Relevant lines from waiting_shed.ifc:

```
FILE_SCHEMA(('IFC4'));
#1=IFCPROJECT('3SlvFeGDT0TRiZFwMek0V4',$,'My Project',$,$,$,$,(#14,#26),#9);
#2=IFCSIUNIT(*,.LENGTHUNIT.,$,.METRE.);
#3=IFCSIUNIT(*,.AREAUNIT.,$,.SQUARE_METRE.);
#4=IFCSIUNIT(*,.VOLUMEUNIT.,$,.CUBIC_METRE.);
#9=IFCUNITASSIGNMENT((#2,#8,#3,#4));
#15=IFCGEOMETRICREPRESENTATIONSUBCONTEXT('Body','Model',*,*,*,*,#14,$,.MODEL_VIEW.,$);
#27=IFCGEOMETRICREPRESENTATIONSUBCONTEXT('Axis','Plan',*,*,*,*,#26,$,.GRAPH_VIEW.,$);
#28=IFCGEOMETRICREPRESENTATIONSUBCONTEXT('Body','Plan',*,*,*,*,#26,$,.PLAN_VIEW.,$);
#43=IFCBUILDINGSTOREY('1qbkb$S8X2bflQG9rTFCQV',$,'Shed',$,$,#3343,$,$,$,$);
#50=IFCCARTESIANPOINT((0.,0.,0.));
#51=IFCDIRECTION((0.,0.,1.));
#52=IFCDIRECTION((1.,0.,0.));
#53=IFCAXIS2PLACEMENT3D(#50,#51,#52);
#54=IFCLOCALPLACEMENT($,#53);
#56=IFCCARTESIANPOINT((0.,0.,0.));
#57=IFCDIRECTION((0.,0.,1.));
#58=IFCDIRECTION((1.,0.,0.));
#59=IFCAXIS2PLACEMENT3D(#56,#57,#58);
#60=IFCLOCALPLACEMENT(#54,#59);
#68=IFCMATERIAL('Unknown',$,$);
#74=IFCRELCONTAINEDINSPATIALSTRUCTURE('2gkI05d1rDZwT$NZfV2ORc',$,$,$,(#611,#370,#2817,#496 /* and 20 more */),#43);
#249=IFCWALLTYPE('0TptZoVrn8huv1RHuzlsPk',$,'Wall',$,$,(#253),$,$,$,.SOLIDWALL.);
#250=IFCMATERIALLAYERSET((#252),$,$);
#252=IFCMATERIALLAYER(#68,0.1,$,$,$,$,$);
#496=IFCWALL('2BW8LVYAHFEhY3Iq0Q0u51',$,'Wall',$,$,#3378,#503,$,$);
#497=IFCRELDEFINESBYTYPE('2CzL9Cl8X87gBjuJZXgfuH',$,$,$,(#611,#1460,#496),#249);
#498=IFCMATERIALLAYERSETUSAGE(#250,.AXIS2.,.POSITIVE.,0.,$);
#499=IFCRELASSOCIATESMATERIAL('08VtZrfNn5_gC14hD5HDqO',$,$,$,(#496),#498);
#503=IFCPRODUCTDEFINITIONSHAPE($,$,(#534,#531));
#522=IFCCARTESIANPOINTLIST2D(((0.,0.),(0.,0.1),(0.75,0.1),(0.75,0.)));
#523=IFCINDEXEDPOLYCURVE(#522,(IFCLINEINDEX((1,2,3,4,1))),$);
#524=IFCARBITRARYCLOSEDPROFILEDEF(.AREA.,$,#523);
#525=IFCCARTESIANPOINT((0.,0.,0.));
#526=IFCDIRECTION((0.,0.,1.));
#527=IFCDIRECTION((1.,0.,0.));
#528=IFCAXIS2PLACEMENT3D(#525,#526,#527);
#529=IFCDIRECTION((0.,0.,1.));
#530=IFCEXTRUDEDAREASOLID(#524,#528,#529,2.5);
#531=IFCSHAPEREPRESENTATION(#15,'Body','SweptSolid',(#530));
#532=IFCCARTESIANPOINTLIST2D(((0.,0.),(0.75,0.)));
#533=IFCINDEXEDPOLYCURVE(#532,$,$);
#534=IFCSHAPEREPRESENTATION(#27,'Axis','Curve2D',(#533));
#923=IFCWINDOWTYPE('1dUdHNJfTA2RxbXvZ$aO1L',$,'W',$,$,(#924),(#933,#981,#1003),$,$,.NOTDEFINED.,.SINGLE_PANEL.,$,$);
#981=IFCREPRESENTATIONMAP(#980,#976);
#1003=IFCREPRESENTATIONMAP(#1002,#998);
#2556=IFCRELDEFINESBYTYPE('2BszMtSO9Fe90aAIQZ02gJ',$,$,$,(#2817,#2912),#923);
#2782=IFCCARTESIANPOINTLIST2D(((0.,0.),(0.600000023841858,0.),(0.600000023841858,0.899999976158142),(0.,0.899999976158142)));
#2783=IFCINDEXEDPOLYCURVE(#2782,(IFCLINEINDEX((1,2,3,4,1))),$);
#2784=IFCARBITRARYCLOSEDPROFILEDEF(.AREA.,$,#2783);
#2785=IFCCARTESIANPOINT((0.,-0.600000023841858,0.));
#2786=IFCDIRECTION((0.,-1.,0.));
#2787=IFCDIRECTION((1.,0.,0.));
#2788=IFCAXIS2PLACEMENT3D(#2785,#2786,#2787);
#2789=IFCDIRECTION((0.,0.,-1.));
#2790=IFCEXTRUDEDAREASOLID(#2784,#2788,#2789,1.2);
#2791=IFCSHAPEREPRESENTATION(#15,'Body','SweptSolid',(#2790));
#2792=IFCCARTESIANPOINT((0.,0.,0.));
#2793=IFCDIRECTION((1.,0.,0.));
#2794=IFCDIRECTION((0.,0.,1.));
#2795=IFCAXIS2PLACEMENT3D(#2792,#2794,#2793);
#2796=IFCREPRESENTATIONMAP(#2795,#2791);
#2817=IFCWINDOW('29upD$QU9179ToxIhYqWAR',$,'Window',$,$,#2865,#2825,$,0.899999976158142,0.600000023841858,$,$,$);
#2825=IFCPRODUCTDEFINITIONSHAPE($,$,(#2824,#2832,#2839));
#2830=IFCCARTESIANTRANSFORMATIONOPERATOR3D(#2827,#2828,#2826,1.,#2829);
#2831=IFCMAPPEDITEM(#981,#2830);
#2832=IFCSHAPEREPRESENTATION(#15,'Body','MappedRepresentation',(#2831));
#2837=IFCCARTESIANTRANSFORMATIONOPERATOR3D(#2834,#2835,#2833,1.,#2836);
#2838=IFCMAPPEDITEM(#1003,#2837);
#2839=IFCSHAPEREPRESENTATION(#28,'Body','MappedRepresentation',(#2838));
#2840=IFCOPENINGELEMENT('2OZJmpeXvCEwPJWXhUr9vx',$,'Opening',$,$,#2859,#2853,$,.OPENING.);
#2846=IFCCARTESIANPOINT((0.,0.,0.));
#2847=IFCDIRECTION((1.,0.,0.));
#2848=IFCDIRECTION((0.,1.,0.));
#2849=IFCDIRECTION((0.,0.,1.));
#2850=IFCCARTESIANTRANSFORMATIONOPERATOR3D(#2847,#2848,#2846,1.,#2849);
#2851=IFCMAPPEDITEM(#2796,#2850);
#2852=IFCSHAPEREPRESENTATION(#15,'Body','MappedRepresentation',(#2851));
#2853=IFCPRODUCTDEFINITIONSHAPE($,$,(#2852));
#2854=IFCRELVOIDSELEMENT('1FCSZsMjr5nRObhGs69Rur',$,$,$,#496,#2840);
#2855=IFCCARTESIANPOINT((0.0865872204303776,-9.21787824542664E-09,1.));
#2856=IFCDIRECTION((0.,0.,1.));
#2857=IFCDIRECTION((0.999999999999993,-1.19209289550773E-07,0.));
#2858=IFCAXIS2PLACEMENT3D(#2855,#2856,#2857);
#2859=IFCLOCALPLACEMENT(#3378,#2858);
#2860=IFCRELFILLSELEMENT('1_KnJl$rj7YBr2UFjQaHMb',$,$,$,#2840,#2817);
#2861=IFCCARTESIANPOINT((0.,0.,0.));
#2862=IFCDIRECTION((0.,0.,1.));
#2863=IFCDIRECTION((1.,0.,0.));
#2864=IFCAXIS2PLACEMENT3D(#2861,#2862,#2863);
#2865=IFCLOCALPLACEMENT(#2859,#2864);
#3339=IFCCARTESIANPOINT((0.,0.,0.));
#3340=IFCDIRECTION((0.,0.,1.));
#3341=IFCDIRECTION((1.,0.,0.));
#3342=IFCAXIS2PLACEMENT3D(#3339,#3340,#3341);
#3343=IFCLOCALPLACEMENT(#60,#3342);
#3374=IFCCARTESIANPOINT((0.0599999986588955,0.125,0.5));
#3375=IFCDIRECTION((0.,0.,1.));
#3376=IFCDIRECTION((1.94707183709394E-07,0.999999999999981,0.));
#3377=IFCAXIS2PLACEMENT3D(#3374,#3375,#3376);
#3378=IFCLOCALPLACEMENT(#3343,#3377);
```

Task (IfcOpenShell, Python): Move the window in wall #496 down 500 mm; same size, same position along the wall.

```python
import numpy as np
import ifcopenshell
import ifcopenshell.api.geometry
import ifcopenshell.util.placement
import ifcopenshell.util.unit

model = ifcopenshell.open("waiting_shed.ifc")
unit_scale = ifcopenshell.util.unit.calculate_unit_scale(model)

window = model.by_id(2817)
opening = window.FillsVoids[0].RelatingOpeningElement
dz = -0.5

shift = np.array([0.0, 0.0, dz])
# The window is placed relative to its opening, so it follows when the opening moves.
matrix = ifcopenshell.util.placement.get_local_placement(opening.ObjectPlacement)
matrix[:3, 3] += shift
ifcopenshell.api.geometry.edit_object_placement(
    model, product=opening, matrix=matrix, is_si=False, should_transform_children=True
)

print(f"moved by {dz * unit_scale:+.3f} m")

model.write("waiting_shed_updated.ifc")
```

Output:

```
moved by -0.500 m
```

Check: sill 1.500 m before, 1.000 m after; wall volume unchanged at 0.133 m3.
